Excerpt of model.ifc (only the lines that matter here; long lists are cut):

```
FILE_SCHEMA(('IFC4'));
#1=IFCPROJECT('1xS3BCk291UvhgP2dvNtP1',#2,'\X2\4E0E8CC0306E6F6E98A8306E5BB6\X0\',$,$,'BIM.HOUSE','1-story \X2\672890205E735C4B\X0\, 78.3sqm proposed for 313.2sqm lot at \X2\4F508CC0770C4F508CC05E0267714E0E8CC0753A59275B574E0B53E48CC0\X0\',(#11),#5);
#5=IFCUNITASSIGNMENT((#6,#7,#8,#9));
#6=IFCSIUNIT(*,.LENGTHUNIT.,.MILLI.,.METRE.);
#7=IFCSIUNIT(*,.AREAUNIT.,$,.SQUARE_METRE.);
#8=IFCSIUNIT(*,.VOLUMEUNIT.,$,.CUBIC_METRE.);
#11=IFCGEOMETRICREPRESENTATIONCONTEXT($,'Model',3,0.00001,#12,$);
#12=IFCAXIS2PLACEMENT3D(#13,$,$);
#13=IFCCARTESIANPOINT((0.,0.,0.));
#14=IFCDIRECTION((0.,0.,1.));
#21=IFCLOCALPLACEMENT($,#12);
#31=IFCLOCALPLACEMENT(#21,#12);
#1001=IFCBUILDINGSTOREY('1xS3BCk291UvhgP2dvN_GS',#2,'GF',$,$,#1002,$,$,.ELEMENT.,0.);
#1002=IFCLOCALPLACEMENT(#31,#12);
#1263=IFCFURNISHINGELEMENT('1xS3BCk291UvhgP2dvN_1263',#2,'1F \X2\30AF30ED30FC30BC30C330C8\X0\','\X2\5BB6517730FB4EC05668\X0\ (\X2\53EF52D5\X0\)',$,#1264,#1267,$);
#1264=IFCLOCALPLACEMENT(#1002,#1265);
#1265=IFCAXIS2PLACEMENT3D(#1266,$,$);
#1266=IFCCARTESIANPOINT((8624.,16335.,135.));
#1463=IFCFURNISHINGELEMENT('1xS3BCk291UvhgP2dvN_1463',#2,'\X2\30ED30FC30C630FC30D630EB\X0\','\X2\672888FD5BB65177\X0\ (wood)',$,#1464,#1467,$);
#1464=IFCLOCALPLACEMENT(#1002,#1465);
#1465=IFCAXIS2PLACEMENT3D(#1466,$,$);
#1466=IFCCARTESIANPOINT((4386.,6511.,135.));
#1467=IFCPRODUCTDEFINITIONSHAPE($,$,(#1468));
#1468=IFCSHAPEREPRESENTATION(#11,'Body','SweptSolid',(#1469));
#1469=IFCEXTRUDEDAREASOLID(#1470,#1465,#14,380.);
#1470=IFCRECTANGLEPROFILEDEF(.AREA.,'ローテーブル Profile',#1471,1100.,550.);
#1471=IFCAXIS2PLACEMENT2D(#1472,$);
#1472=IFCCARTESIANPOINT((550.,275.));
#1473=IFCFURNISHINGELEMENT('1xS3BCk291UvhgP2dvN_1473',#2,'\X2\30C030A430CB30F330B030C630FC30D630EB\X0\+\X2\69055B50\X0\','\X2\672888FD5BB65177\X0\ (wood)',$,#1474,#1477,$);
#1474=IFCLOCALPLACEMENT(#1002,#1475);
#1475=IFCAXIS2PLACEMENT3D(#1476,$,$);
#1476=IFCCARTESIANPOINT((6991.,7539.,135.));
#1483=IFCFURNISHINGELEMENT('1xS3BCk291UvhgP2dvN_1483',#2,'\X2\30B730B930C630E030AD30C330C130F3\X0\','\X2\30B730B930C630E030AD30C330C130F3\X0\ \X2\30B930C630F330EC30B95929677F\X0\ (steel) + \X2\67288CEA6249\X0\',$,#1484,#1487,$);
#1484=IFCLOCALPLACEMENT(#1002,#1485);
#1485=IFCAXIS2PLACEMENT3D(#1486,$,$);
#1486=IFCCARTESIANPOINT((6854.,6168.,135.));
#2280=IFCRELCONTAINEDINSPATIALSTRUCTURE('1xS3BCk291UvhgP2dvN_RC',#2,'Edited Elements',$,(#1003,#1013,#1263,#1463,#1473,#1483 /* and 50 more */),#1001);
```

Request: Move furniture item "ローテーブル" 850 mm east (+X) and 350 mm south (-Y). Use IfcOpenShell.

```python
import ifcopenshell
import ifcopenshell.api.geometry
import ifcopenshell.util.placement
import ifcopenshell.util.unit

model = ifcopenshell.open("model.ifc")
unit_scale = ifcopenshell.util.unit.calculate_unit_scale(model)

item = model.by_guid("1xS3BCk291UvhgP2dvN_1463")
matrix = ifcopenshell.util.placement.get_local_placement(item.ObjectPlacement)
matrix[0, 3] += 0.85 / unit_scale
matrix[1, 3] -= 0.35 / unit_scale
ifcopenshell.api.geometry.edit_object_placement(model, product=item, matrix=matrix, is_si=False)

print(ifcopenshell.util.placement.get_local_placement(item.ObjectPlacement).round(3) + 0.0)

model.write("model_rev.ifc")
```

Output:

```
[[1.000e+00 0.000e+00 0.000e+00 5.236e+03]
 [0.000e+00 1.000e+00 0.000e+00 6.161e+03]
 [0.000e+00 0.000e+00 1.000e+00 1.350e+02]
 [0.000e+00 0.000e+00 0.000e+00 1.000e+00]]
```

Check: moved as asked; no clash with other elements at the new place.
